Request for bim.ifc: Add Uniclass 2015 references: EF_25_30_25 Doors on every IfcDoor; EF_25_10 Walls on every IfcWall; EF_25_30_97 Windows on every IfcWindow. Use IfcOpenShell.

First a look at what the model holds.

```python
import ifcopenshell

model = ifcopenshell.open("bim.ifc")
print(model.schema)
print("classifications:", [c.Name for c in model.by_type("IfcClassification")])
for ifc_class in ("IfcDoor", "IfcRoof", "IfcStair", "IfcWall", "IfcWindow"):
    print(ifc_class, len(model.by_type(ifc_class)))
```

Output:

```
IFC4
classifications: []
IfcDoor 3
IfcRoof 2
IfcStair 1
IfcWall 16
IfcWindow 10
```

```python
import ifcopenshell
import ifcopenshell.api.classification

model = ifcopenshell.open("bim.ifc")

system = ifcopenshell.api.classification.add_classification(model, classification="Uniclass 2015")

codes = {
    "IfcDoor": ("EF_25_30_25", "Doors"),
    "IfcWall": ("EF_25_10", "Walls"),
    "IfcWindow": ("EF_25_30_97", "Windows"),
}
for ifc_class, (code, name) in codes.items():
    products = model.by_type(ifc_class)
    ifcopenshell.api.classification.add_reference(
        model, products=products, classification=system, identification=code, name=name
    )
    print(code, len(products))

model.write("bim_updated.ifc")
```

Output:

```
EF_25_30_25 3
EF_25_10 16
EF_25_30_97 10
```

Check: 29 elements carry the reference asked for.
